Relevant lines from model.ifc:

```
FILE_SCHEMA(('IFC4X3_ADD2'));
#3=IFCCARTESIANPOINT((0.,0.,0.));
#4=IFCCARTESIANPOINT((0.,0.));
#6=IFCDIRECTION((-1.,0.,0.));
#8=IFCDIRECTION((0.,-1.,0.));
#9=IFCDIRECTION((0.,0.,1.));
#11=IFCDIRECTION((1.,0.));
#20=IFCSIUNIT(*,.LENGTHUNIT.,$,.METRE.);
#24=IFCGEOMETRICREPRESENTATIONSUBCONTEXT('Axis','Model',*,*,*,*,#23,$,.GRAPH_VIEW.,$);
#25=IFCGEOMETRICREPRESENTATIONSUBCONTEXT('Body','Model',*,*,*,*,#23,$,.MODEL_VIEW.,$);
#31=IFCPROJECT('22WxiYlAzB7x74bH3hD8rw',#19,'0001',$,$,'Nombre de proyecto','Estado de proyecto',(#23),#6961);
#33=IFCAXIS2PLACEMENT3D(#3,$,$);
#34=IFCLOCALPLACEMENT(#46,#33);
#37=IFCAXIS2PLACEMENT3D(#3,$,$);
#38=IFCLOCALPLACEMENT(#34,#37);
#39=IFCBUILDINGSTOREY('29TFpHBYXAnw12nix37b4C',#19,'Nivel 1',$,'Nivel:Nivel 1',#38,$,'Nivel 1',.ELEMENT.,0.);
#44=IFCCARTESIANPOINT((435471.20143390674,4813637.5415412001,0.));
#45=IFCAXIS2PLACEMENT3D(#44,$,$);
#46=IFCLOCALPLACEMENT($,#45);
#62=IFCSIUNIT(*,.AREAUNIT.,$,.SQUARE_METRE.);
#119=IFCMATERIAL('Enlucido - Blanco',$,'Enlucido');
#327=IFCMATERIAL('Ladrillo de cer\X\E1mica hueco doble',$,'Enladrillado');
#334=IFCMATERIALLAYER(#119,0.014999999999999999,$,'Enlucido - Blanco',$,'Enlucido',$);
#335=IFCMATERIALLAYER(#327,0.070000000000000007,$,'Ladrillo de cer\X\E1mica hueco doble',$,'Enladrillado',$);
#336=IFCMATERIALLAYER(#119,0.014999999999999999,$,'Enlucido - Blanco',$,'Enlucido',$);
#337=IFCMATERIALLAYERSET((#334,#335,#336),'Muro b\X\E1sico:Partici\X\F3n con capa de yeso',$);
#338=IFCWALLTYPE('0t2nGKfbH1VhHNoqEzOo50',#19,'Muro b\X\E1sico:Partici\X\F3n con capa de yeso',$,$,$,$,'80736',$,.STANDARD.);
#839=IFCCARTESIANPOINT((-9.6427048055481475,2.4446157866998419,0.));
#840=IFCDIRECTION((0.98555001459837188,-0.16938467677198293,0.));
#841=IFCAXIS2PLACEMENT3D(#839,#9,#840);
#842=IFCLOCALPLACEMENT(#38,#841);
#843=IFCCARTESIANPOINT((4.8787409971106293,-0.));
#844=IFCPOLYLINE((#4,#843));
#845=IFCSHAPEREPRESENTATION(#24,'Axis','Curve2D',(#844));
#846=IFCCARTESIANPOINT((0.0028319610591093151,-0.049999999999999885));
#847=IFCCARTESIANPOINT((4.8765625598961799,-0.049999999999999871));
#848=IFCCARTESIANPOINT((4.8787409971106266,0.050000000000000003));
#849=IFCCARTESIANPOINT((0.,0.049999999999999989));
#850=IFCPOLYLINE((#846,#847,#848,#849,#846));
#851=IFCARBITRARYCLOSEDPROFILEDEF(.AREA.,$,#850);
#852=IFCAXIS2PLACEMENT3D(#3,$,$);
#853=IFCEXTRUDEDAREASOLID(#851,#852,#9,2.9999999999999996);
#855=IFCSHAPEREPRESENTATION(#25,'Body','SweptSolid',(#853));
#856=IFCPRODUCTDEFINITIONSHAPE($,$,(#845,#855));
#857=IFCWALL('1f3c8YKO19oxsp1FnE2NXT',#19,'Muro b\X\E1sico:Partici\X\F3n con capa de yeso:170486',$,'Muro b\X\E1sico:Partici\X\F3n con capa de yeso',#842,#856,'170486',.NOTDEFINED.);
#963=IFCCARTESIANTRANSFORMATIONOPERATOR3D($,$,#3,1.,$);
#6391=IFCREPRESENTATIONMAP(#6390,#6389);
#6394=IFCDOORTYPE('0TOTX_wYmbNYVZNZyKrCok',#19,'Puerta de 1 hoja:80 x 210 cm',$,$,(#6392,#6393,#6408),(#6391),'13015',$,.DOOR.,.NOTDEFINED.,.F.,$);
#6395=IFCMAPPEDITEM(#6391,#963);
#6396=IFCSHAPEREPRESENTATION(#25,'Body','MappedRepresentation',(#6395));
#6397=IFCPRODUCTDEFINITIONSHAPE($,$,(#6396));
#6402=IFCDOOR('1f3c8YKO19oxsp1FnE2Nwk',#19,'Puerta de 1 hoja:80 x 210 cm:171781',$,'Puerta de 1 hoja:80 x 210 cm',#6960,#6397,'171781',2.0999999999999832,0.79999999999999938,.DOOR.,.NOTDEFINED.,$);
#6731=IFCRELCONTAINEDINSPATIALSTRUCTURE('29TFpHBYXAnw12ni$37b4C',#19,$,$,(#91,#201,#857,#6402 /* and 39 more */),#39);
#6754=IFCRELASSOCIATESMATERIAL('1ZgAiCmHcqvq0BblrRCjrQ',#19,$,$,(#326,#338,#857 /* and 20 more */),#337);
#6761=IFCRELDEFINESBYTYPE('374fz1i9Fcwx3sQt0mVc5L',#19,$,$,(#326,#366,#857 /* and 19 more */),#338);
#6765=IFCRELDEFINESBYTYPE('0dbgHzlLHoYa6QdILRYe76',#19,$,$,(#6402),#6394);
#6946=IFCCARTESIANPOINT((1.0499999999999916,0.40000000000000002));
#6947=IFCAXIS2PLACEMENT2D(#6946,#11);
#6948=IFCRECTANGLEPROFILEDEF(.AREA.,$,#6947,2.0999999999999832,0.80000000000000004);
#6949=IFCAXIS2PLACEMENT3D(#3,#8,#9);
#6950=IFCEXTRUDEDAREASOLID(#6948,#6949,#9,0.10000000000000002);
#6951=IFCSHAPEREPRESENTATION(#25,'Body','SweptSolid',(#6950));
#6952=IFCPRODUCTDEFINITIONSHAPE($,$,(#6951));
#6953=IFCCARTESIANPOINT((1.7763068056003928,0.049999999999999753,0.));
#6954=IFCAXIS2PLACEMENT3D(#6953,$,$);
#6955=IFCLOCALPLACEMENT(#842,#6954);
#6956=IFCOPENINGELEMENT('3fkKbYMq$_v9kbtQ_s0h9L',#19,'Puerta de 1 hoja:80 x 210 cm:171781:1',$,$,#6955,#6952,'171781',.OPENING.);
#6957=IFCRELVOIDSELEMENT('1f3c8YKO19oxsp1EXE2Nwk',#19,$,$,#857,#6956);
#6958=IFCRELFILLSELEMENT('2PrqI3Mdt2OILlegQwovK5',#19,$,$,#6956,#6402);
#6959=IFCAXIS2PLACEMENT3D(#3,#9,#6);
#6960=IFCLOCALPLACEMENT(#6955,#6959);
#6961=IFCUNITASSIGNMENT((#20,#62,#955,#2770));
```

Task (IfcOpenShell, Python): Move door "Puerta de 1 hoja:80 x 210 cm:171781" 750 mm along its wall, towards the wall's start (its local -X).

```python
import ifcopenshell
import ifcopenshell.api.geometry
import ifcopenshell.util.placement

model = ifcopenshell.open("model.ifc")

door = model.by_guid("1f3c8YKO19oxsp1FnE2Nwk")
opening = door.FillsVoids[0].RelatingOpeningElement
wall = opening.VoidsElements[0].RelatingBuildingElement

wall_matrix = ifcopenshell.util.placement.get_local_placement(wall.ObjectPlacement)
shift = wall_matrix[:3, 0] * -0.75
before = ifcopenshell.util.placement.get_local_placement(door.ObjectPlacement)[:3, 3].copy()

# The door is placed relative to its opening, so it follows when the opening moves.
matrix = ifcopenshell.util.placement.get_local_placement(opening.ObjectPlacement)
matrix[:3, 3] += shift
ifcopenshell.api.geometry.edit_object_placement(
    model, product=opening, matrix=matrix, is_si=False, should_transform_children=True
)

after = ifcopenshell.util.placement.get_local_placement(door.ObjectPlacement)[:3, 3]
print("door moved by", (after - before).round(3) + 0.0)

model.write("model_rev.ifc")
```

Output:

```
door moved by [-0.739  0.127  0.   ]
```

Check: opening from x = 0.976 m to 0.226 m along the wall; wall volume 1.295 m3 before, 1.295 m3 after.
